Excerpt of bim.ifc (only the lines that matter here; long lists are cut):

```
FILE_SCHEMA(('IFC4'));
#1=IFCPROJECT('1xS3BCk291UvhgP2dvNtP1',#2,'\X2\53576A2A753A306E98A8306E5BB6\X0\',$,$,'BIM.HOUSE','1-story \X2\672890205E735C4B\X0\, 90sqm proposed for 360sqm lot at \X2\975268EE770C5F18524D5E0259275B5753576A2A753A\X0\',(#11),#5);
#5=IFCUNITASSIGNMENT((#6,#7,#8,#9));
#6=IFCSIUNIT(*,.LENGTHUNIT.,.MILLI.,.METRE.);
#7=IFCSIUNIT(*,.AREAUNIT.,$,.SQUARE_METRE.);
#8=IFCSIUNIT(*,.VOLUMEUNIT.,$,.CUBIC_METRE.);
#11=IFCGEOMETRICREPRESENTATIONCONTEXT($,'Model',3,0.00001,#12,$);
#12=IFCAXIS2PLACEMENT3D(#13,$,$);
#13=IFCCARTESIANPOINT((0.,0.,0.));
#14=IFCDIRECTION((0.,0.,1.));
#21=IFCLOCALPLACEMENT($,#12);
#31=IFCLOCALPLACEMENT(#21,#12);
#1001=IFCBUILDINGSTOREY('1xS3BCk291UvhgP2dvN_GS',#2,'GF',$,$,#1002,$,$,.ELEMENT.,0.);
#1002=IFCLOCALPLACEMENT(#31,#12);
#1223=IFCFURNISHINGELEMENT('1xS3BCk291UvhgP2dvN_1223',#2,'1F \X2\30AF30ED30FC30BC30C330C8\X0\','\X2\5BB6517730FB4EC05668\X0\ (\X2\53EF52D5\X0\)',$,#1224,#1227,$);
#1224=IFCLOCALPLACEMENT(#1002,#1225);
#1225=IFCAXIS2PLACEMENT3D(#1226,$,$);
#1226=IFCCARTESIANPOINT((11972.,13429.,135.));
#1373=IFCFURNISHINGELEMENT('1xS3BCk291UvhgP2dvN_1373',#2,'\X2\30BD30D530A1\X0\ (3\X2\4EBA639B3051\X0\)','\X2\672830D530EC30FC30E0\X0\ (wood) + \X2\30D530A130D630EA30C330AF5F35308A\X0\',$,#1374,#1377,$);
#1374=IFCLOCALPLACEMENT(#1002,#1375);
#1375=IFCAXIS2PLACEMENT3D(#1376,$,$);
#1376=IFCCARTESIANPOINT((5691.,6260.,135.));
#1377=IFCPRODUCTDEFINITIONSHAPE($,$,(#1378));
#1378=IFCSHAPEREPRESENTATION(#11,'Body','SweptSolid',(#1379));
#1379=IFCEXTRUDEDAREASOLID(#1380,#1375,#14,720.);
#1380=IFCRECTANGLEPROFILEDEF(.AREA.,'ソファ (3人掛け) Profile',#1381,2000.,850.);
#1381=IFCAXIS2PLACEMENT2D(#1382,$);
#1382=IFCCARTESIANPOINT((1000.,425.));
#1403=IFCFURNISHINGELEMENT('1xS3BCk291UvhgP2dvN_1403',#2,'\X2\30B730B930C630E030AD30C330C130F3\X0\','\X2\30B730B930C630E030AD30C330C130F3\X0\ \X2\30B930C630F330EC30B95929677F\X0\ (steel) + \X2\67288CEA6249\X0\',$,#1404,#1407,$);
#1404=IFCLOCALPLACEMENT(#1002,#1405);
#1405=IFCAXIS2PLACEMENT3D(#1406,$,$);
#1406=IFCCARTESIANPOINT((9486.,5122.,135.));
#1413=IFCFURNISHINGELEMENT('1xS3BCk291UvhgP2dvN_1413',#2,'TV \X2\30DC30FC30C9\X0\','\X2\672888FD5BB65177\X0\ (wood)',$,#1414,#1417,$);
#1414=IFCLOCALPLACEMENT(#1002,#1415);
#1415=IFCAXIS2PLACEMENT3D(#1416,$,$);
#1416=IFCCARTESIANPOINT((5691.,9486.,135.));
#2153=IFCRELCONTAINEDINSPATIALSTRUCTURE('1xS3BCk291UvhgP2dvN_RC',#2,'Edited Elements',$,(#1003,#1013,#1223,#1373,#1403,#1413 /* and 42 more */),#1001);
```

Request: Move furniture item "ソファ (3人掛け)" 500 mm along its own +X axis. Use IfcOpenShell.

```python
import ifcopenshell
import ifcopenshell.api.geometry
import ifcopenshell.util.placement

model = ifcopenshell.open("bim.ifc")

item = model.by_id(1373)
matrix = ifcopenshell.util.placement.get_local_placement(item.ObjectPlacement)
matrix[:3, 3] += matrix[:3, 0] * 500.0
ifcopenshell.api.geometry.edit_object_placement(model, product=item, matrix=matrix, is_si=False)

print(ifcopenshell.util.placement.get_local_placement(item.ObjectPlacement).round(3) + 0.0)

model.write("bim_rev.ifc")
```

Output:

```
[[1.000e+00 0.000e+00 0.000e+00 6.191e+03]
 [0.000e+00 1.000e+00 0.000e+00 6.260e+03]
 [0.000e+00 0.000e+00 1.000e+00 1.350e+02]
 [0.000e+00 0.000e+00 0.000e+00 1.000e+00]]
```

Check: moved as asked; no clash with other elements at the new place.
